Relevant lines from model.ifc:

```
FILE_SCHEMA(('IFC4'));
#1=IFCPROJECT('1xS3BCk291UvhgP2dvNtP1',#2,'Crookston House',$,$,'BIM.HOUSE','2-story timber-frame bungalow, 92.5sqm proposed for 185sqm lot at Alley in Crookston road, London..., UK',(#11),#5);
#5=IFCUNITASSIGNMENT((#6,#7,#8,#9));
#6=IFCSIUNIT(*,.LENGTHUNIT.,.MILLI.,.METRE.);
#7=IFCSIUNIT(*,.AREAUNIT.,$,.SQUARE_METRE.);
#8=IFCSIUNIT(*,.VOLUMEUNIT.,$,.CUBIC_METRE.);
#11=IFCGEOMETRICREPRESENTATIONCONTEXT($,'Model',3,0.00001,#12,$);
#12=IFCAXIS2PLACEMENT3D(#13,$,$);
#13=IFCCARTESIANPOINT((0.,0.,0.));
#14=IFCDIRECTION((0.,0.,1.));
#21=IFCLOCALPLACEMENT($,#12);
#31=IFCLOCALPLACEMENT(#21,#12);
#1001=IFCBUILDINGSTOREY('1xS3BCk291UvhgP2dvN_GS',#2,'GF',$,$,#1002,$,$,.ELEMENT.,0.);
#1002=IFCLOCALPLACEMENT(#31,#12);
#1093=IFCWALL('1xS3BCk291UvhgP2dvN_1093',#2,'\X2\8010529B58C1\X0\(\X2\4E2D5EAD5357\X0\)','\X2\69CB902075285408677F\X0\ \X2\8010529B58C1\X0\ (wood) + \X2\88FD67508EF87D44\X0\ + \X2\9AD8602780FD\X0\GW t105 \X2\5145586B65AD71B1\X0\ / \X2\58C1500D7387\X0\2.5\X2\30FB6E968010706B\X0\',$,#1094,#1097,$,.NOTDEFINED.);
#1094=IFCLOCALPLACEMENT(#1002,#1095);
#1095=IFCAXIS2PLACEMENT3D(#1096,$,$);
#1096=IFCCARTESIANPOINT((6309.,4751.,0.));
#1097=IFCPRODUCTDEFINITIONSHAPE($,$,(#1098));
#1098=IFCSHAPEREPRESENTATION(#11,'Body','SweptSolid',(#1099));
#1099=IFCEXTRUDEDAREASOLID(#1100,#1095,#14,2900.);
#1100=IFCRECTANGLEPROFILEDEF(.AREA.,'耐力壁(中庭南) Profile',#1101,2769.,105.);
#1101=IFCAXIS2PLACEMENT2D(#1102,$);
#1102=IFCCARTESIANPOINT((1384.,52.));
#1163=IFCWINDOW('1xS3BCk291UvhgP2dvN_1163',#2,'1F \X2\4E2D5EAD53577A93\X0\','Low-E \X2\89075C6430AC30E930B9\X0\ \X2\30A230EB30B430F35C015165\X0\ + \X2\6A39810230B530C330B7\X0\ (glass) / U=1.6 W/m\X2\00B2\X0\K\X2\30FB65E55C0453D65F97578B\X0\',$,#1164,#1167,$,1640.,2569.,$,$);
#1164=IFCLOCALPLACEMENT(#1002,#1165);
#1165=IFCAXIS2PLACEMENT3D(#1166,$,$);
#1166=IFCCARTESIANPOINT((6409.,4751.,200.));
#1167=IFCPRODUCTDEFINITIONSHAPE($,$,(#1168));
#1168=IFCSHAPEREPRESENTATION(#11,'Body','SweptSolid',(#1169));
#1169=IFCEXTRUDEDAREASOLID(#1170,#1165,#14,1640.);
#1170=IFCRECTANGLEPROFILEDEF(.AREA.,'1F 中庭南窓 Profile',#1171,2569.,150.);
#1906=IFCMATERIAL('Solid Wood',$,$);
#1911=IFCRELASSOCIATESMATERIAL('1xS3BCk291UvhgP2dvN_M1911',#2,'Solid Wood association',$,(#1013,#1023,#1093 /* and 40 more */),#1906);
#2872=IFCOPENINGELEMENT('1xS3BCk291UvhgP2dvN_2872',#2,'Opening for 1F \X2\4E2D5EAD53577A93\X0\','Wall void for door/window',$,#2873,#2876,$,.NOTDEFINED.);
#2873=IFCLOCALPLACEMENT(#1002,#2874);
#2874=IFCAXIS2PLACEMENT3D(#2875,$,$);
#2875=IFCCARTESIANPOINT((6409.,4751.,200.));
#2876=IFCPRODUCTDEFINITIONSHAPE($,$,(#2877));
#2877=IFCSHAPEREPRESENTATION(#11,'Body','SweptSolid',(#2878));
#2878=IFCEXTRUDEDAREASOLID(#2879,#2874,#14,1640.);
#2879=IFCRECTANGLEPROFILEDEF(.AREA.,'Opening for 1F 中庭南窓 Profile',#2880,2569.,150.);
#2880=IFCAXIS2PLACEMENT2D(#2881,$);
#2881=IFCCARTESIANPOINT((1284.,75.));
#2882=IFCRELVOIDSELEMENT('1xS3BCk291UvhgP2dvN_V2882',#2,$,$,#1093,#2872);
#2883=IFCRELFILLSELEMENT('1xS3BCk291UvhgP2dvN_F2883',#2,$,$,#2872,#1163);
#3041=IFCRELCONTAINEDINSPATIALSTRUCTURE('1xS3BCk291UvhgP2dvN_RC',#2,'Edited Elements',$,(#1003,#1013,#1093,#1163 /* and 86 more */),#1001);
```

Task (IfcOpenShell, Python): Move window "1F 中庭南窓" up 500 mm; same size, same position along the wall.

```python
import numpy as np
import ifcopenshell
import ifcopenshell.api.geometry
import ifcopenshell.util.placement
import ifcopenshell.util.unit

model = ifcopenshell.open("model.ifc")
unit_scale = ifcopenshell.util.unit.calculate_unit_scale(model)

window = model.by_guid("1xS3BCk291UvhgP2dvN_1163")
opening = window.FillsVoids[0].RelatingOpeningElement
dz = 500.0

shift = np.array([0.0, 0.0, dz])
# The window is not placed relative to its opening, so move both.
for product in (opening, window):
    matrix = ifcopenshell.util.placement.get_local_placement(product.ObjectPlacement)
    matrix[:3, 3] += shift
    ifcopenshell.api.geometry.edit_object_placement(model, product=product, matrix=matrix, is_si=False)

print(f"moved by {dz * unit_scale:+.3f} m")

model.write("model_updated.ifc")
```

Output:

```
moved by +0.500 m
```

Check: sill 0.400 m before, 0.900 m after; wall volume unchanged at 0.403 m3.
